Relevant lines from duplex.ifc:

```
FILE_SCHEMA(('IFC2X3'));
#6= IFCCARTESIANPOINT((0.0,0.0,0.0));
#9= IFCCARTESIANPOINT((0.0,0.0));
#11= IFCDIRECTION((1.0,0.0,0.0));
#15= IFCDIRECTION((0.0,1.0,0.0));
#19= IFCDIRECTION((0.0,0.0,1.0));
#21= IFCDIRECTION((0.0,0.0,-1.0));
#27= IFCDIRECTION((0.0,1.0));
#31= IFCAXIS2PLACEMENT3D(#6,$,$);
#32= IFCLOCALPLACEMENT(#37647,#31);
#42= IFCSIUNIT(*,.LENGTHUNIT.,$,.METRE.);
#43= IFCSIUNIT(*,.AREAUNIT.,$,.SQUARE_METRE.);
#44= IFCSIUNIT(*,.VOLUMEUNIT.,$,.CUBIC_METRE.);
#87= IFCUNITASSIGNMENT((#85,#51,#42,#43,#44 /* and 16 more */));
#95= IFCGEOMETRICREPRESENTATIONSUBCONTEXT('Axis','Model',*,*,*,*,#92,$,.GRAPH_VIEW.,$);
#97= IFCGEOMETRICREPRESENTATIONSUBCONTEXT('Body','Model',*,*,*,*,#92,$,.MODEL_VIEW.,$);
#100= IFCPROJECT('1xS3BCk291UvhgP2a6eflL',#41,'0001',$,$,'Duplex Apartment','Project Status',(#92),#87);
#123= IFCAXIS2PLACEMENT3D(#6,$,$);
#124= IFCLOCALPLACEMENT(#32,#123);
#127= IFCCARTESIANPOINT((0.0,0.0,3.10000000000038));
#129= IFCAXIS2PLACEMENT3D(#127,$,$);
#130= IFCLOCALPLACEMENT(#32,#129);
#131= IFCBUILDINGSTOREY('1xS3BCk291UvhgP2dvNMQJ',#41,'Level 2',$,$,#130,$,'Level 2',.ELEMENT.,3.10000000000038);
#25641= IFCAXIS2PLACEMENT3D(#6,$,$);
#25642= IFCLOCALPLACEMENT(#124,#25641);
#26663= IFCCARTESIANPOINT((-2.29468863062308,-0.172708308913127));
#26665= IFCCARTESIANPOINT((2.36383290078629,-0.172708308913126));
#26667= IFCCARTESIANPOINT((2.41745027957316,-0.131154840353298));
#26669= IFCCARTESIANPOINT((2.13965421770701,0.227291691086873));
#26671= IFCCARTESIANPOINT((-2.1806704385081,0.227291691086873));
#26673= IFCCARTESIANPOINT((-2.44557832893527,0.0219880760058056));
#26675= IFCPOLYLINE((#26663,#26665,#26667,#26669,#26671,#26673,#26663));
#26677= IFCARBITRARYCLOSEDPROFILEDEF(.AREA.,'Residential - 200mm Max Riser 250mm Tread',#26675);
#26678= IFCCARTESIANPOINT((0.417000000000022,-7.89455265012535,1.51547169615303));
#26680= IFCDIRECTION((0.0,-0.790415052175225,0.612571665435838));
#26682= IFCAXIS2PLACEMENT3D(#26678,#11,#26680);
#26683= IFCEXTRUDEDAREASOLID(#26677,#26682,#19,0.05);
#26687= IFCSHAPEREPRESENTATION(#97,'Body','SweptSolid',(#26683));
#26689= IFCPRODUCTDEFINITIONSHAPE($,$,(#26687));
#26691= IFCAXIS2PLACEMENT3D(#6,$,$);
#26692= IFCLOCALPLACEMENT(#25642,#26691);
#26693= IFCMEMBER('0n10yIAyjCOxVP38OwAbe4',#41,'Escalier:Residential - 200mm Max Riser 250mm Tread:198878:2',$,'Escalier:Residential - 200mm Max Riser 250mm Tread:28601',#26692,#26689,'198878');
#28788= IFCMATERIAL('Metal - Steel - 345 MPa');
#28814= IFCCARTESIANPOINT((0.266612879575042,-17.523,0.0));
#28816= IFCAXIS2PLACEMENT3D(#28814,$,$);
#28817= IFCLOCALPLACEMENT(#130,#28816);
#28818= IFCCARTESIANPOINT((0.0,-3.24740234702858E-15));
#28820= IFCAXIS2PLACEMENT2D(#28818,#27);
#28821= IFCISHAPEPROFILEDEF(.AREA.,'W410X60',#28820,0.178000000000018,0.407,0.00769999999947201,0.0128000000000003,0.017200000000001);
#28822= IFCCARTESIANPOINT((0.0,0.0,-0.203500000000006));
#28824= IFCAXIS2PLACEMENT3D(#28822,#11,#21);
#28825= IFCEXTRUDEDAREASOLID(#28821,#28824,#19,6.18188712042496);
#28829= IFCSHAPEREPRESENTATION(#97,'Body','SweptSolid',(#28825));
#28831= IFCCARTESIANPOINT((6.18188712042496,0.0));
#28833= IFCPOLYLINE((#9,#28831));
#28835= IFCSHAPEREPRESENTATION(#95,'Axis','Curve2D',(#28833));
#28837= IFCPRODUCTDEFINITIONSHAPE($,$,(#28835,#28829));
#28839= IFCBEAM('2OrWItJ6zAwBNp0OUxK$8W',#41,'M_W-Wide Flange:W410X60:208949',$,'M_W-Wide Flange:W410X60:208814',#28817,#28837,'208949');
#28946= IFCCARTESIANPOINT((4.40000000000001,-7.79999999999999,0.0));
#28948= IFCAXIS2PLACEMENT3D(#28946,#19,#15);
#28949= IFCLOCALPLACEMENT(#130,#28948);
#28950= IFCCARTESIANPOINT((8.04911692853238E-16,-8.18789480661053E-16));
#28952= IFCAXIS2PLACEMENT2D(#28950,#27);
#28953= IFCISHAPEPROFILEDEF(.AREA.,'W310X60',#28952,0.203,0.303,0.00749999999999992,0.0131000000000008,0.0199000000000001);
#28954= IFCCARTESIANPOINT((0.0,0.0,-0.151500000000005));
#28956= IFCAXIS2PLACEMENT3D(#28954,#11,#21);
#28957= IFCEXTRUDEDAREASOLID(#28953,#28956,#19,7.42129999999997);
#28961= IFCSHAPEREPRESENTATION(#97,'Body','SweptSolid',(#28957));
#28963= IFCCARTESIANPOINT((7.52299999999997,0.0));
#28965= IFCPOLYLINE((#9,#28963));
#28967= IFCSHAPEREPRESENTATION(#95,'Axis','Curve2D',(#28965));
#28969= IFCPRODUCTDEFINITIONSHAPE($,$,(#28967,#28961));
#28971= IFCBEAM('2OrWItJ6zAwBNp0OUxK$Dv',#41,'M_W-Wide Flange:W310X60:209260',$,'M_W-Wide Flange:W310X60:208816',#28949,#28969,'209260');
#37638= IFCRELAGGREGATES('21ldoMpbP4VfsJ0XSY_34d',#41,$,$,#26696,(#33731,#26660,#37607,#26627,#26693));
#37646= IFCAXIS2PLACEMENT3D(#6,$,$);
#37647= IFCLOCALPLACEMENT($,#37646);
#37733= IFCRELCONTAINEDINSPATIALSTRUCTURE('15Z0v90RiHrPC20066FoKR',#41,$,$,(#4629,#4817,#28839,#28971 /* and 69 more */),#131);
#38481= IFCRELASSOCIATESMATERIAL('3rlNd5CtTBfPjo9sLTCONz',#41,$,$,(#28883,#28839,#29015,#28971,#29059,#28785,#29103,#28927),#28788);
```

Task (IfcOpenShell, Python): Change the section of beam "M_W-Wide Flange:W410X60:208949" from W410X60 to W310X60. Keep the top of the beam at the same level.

```python
import ifcopenshell
import ifcopenshell.util.element
import ifcopenshell.util.representation

model = ifcopenshell.open("duplex.ifc")

member = model.by_guid("2OrWItJ6zAwBNp0OUxK$8W")
source = next(p for p in model.by_type("IfcIShapeProfileDef") if p.ProfileName == "W310X60")

body = ifcopenshell.util.representation.get_representation(member, "Model", "Body")
solid = body.Items[0]
old_profile = solid.SweptArea

# Copy the section's sizes but keep this member's own profile position.
profile = ifcopenshell.util.element.copy(model, source)
# Profiles are centred, so shift by half the change in depth to hold the top.
shift = (old_profile.OverallDepth - profile.OverallDepth) / 2
x, y = old_profile.Position.Location.Coordinates
up = (-1.0, 0.0)  # upwards, in the solid's own plane
location = model.createIfcCartesianPoint((x + up[0] * shift, y + up[1] * shift))
profile.Position = model.createIfcAxis2Placement2D(location, old_profile.Position.RefDirection)
solid.SweptArea = profile
if not model.get_total_inverses(old_profile):
    ifcopenshell.util.element.remove_deep2(model, old_profile)
member.Name = member.Name.replace("W410X60", "W310X60")
member.ObjectType = member.ObjectType.replace("W410X60", "W310X60")

print(solid.SweptArea)

model.write("duplex_rev.ifc")
```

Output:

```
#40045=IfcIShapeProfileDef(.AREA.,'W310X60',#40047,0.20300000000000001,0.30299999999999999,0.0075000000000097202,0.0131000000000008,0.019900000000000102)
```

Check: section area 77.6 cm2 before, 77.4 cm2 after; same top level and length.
